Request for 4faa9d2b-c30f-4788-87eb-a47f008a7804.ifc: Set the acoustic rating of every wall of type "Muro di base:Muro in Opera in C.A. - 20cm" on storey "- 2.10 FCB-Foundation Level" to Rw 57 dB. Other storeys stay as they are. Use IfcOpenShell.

First a look at what the model holds.

```python
import ifcopenshell
import ifcopenshell.util.element

model = ifcopenshell.open("4faa9d2b-c30f-4788-87eb-a47f008a7804.ifc")
print(model.schema)
storey = next(s for s in model.by_type("IfcBuildingStorey") if s.Name == "- 2.10 FCB-Foundation Level")
walls = [e for e in ifcopenshell.util.element.get_decomposition(storey) if e.is_a("IfcWall")]
seen = {}
for e in walls:
    element_type = ifcopenshell.util.element.get_type(e)
    key = (element_type.Name if element_type != e and element_type else None, ifcopenshell.util.element.get_pset(e, "Pset_WallCommon", "AcousticRating"))
    seen[key] = seen.get(key, 0) + 1
for (name, value), count in sorted(seen.items(), key=str):
    print(count, "x", name, "|", value)
```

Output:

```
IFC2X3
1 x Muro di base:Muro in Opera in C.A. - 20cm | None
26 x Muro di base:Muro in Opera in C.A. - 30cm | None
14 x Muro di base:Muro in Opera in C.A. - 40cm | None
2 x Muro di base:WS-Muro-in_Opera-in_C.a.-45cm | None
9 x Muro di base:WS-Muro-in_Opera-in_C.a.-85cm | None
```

```python
import ifcopenshell
import ifcopenshell.api.pset
import ifcopenshell.util.element

model = ifcopenshell.open("4faa9d2b-c30f-4788-87eb-a47f008a7804.ifc")

storey = next(s for s in model.by_type("IfcBuildingStorey") if s.Name == "- 2.10 FCB-Foundation Level")
walls = [e for e in ifcopenshell.util.element.get_decomposition(storey) if e.is_a("IfcWall")]

count = 0
for e in walls:
    element_type = ifcopenshell.util.element.get_type(e)
    if element_type in (None, e) or element_type.Name != "Muro di base:Muro in Opera in C.A. - 20cm":
        continue
    # add_pset returns the element's existing set when there is one.
    pset = ifcopenshell.api.pset.add_pset(model, product=e, name="Pset_WallCommon")
    ifcopenshell.api.pset.edit_pset(model, pset=pset, properties={"AcousticRating": "Rw 57 dB"})
    count += 1

print(count, "walls updated")

model.write("4faa9d2b-c30f-4788-87eb-a47f008a7804-out.ifc")
```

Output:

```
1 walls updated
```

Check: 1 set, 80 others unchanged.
